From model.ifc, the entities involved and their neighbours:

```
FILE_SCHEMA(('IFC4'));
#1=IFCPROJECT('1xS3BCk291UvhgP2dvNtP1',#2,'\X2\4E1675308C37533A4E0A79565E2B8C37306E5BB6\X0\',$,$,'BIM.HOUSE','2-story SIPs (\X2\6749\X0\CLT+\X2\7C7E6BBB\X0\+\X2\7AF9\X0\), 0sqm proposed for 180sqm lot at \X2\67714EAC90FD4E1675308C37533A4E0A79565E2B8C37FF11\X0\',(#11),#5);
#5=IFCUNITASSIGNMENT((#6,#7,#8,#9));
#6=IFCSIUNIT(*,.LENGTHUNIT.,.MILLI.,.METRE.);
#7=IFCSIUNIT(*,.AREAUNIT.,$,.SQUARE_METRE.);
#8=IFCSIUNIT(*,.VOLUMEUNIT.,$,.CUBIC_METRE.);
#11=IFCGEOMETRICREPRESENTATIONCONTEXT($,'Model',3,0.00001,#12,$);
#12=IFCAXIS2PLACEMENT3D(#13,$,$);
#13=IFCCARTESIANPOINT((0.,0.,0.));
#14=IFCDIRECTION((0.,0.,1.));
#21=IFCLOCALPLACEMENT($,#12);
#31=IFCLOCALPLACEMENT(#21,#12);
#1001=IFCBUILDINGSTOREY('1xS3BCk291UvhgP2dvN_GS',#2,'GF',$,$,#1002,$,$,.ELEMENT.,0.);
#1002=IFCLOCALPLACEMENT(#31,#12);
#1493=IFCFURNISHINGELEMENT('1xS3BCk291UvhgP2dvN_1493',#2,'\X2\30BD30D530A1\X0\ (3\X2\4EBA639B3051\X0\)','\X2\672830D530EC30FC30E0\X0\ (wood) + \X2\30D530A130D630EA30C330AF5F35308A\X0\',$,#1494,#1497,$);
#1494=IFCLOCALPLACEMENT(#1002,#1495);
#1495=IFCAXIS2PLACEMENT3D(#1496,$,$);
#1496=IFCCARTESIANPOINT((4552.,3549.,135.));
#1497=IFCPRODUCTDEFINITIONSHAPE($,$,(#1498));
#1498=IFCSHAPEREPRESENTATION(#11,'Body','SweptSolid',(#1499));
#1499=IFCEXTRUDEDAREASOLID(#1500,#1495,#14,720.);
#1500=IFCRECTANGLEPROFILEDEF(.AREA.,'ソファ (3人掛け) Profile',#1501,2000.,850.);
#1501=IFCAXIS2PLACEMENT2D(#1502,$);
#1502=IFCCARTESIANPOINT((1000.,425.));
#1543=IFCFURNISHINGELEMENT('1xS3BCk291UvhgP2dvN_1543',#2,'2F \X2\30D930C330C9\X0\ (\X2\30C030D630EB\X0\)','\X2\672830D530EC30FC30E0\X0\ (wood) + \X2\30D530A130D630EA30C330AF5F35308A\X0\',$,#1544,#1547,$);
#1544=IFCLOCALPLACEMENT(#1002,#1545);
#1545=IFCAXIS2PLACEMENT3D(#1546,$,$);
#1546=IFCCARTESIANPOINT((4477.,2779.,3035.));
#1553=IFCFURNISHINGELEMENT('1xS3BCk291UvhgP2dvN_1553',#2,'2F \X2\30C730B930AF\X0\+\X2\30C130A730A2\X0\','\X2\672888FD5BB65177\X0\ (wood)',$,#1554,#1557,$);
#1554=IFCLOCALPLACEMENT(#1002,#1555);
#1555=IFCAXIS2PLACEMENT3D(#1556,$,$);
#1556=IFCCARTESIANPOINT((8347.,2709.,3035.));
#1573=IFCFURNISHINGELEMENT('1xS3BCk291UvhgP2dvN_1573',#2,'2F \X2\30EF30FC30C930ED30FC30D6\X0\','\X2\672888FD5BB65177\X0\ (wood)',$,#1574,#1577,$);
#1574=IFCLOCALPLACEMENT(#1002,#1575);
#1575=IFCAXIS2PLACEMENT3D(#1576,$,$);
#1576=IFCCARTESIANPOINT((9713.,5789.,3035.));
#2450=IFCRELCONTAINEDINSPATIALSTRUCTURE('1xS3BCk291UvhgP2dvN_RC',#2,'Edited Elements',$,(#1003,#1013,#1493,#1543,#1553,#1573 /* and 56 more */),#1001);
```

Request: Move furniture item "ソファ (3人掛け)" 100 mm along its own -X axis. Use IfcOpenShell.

```python
import ifcopenshell
import ifcopenshell.api.geometry
import ifcopenshell.util.placement
import ifcopenshell.util.unit

model = ifcopenshell.open("model.ifc")
unit_scale = ifcopenshell.util.unit.calculate_unit_scale(model)

item = model.by_guid("1xS3BCk291UvhgP2dvN_1493")
matrix = ifcopenshell.util.placement.get_local_placement(item.ObjectPlacement)
matrix[:3, 3] -= matrix[:3, 0] * 0.1 / unit_scale
ifcopenshell.api.geometry.edit_object_placement(model, product=item, matrix=matrix, is_si=False)

print(ifcopenshell.util.placement.get_local_placement(item.ObjectPlacement).round(3) + 0.0)

model.write("model_v2.ifc")
```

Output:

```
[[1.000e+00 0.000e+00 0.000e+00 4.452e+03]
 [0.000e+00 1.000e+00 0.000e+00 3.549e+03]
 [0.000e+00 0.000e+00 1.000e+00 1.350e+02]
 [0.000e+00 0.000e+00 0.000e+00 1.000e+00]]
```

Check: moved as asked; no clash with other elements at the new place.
